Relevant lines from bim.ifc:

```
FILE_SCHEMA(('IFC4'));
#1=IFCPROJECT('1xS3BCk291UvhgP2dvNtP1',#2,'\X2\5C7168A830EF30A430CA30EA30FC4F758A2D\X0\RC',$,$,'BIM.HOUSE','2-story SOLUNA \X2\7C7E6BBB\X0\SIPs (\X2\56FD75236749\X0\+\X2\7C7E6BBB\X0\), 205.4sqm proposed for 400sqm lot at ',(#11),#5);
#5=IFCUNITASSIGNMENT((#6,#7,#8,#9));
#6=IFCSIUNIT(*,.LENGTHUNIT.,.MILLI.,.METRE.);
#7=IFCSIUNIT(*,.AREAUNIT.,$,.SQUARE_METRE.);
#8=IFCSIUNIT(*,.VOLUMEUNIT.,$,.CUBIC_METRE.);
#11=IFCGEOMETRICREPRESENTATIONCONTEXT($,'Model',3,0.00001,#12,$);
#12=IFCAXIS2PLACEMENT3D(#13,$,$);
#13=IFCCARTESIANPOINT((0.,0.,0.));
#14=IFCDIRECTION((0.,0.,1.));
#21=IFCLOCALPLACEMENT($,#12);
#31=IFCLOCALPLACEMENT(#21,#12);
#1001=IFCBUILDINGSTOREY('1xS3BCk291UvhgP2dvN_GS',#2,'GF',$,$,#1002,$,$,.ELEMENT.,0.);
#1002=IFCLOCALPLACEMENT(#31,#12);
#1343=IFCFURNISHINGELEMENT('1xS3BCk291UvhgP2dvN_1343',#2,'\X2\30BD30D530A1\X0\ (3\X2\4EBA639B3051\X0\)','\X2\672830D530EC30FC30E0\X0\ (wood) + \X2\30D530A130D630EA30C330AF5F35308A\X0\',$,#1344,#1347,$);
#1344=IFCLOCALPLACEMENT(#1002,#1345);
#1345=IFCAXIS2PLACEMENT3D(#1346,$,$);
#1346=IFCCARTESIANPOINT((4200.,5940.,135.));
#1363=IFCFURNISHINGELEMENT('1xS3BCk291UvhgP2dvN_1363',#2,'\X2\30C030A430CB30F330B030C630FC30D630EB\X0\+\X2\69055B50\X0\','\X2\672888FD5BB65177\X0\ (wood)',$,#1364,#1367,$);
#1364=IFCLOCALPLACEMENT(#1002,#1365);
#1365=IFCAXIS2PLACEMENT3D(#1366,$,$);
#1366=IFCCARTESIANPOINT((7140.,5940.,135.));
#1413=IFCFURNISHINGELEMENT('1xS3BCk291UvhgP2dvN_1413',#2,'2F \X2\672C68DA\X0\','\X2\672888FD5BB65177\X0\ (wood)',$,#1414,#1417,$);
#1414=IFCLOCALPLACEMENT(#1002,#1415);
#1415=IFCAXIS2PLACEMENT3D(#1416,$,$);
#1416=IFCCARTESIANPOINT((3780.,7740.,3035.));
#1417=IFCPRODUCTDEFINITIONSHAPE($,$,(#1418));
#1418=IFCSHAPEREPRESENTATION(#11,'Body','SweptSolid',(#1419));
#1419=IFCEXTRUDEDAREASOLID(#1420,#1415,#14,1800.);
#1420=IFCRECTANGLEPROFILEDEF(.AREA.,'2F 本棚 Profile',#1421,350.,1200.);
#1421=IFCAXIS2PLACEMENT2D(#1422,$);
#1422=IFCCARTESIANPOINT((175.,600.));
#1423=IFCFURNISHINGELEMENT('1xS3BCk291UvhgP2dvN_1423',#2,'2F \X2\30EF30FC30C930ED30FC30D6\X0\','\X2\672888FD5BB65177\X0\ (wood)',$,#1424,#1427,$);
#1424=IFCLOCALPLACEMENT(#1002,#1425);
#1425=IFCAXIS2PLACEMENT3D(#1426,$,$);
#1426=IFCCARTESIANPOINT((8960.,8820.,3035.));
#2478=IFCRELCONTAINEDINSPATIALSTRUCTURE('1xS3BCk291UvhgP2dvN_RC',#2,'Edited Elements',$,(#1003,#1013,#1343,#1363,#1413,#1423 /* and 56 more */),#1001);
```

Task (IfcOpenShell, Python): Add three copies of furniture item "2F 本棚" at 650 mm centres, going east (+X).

```python
import numpy as np
import ifcopenshell
import ifcopenshell.api.geometry
import ifcopenshell.api.root
import ifcopenshell.util.element
import ifcopenshell.util.placement

model = ifcopenshell.open("bim.ifc")


def reuse_history(source, copy):
    """copy_class also copies each property set's owner history, people and application; keep the originals."""
    for rel in copy.IsDefinedBy:
        if rel.is_a("IfcRelDefinesByProperties") and (history := rel.RelatingPropertyDefinition.OwnerHistory):
            rel.RelatingPropertyDefinition.OwnerHistory = source.OwnerHistory
            ifcopenshell.util.element.remove_deep2(model, history)


source = model.by_guid("1xS3BCk291UvhgP2dvN_1413")
base = ifcopenshell.util.placement.get_local_placement(source.ObjectPlacement)
step = np.array([1.0, 0.0, 0.0]) * 650.0

for i in range(1, 4):
    copy = ifcopenshell.api.root.copy_class(model, product=source)
    copy.Representation = ifcopenshell.util.element.copy_deep(
        model, source.Representation, exclude=["IfcGeometricRepresentationContext", "IfcRepresentationMap"]
    )
    reuse_history(source, copy)
    matrix = base.copy()
    matrix[:3, 3] += i * step
    print("added at", matrix[:3, 3].round(3) + 0.0)
    ifcopenshell.api.geometry.edit_object_placement(model, product=copy, matrix=matrix, is_si=False)

model.write("bim_rev.ifc")
```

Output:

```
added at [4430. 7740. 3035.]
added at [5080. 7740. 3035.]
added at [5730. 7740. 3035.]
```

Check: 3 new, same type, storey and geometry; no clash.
